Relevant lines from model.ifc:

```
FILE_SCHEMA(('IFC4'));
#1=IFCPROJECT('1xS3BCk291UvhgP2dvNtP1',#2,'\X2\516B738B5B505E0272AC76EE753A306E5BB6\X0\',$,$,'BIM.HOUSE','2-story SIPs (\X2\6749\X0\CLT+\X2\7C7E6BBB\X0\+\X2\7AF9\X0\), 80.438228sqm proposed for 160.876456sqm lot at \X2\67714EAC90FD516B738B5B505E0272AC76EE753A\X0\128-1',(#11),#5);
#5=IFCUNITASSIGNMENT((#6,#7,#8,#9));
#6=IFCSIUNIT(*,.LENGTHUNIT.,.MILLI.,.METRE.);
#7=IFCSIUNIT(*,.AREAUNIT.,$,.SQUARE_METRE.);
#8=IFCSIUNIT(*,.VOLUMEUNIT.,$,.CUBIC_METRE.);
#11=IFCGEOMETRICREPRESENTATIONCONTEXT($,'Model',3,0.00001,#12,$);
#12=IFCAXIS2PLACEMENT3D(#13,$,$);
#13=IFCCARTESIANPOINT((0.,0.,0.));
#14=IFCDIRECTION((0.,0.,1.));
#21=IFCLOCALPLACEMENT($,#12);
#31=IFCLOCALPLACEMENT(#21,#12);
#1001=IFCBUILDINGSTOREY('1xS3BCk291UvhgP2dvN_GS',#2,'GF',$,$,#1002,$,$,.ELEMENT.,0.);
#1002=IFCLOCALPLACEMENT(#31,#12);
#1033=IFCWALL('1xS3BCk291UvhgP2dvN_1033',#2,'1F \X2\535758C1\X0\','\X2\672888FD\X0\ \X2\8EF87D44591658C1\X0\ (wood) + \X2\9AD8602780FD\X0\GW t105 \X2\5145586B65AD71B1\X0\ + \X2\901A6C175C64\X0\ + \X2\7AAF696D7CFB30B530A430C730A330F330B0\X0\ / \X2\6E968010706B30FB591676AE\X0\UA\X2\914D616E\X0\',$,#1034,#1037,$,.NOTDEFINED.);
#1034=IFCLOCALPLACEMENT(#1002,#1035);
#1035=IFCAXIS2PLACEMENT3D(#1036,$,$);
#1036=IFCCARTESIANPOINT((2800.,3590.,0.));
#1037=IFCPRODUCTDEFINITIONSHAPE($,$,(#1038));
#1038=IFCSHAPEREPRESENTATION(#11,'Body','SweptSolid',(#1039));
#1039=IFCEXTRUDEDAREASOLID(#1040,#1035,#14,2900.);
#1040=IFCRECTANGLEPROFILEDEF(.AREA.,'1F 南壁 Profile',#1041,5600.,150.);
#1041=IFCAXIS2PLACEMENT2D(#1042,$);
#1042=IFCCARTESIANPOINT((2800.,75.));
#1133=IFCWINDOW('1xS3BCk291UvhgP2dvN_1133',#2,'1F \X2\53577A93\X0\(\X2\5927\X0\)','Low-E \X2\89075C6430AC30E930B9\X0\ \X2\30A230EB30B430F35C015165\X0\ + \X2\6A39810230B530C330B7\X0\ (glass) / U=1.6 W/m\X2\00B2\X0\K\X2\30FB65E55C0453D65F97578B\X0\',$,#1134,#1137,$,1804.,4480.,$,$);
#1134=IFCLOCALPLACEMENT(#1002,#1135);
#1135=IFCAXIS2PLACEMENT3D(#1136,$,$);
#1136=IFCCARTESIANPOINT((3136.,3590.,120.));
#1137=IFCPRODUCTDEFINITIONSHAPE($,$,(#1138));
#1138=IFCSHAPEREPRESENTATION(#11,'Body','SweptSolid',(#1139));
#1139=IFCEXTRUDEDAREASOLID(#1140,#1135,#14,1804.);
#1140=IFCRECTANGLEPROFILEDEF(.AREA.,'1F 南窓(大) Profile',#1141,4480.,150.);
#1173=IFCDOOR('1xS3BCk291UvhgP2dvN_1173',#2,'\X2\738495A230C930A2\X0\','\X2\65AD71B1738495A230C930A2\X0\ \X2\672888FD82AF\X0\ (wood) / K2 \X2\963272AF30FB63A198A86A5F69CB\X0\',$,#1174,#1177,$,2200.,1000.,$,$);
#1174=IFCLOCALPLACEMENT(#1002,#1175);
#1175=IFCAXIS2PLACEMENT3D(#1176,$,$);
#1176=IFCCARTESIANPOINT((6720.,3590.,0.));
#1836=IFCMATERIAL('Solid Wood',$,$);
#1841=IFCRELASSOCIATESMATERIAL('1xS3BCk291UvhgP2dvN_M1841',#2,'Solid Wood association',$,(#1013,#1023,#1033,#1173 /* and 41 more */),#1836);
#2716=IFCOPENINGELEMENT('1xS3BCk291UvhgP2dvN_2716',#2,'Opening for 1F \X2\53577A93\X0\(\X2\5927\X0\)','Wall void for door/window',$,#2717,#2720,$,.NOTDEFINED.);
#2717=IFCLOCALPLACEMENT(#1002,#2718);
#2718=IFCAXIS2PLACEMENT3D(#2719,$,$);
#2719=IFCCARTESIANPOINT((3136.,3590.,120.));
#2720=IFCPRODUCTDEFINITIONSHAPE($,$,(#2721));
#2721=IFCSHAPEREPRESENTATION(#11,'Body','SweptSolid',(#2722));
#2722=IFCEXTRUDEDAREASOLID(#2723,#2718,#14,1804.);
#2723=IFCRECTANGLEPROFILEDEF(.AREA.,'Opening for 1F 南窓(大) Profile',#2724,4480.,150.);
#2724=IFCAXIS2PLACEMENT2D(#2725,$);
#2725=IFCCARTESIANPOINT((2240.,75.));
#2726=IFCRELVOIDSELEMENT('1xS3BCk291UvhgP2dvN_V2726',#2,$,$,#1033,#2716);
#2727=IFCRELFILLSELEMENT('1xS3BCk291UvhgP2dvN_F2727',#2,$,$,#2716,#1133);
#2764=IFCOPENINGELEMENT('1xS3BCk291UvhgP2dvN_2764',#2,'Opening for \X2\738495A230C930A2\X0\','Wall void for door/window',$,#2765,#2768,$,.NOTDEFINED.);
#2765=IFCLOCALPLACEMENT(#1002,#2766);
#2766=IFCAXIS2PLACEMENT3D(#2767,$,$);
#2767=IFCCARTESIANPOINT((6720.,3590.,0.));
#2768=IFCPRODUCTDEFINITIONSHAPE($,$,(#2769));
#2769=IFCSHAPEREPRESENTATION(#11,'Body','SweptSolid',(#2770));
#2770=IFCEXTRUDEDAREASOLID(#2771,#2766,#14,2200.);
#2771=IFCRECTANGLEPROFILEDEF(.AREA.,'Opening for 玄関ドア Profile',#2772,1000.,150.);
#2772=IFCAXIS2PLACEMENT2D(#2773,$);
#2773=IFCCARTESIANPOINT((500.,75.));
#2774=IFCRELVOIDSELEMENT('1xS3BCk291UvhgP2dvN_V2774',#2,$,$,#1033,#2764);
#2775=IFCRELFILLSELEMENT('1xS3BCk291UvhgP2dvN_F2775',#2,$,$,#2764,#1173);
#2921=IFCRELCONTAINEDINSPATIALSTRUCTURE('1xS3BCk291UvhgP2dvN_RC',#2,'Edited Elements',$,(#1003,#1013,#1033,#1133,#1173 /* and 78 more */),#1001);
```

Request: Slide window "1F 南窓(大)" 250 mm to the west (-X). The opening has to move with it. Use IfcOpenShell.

```python
import ifcopenshell
import ifcopenshell.api.geometry
import ifcopenshell.util.placement

model = ifcopenshell.open("model.ifc")

window = model.by_id(1133)
opening = window.FillsVoids[0].RelatingOpeningElement
wall = opening.VoidsElements[0].RelatingBuildingElement

wall_matrix = ifcopenshell.util.placement.get_local_placement(wall.ObjectPlacement)
shift = wall_matrix[:3, 0] * -250.0
before = ifcopenshell.util.placement.get_local_placement(window.ObjectPlacement)[:3, 3].copy()

# The window is not placed relative to its opening, so move both.
for product in (opening, window):
    matrix = ifcopenshell.util.placement.get_local_placement(product.ObjectPlacement)
    matrix[:3, 3] += shift
    ifcopenshell.api.geometry.edit_object_placement(model, product=product, matrix=matrix, is_si=False)

after = ifcopenshell.util.placement.get_local_placement(window.ObjectPlacement)[:3, 3]
print("window moved by", (after - before).round(3) + 0.0)

model.write("model_rev.ifc")
```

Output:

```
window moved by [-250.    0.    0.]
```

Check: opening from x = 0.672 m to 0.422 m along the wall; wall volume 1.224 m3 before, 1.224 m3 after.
